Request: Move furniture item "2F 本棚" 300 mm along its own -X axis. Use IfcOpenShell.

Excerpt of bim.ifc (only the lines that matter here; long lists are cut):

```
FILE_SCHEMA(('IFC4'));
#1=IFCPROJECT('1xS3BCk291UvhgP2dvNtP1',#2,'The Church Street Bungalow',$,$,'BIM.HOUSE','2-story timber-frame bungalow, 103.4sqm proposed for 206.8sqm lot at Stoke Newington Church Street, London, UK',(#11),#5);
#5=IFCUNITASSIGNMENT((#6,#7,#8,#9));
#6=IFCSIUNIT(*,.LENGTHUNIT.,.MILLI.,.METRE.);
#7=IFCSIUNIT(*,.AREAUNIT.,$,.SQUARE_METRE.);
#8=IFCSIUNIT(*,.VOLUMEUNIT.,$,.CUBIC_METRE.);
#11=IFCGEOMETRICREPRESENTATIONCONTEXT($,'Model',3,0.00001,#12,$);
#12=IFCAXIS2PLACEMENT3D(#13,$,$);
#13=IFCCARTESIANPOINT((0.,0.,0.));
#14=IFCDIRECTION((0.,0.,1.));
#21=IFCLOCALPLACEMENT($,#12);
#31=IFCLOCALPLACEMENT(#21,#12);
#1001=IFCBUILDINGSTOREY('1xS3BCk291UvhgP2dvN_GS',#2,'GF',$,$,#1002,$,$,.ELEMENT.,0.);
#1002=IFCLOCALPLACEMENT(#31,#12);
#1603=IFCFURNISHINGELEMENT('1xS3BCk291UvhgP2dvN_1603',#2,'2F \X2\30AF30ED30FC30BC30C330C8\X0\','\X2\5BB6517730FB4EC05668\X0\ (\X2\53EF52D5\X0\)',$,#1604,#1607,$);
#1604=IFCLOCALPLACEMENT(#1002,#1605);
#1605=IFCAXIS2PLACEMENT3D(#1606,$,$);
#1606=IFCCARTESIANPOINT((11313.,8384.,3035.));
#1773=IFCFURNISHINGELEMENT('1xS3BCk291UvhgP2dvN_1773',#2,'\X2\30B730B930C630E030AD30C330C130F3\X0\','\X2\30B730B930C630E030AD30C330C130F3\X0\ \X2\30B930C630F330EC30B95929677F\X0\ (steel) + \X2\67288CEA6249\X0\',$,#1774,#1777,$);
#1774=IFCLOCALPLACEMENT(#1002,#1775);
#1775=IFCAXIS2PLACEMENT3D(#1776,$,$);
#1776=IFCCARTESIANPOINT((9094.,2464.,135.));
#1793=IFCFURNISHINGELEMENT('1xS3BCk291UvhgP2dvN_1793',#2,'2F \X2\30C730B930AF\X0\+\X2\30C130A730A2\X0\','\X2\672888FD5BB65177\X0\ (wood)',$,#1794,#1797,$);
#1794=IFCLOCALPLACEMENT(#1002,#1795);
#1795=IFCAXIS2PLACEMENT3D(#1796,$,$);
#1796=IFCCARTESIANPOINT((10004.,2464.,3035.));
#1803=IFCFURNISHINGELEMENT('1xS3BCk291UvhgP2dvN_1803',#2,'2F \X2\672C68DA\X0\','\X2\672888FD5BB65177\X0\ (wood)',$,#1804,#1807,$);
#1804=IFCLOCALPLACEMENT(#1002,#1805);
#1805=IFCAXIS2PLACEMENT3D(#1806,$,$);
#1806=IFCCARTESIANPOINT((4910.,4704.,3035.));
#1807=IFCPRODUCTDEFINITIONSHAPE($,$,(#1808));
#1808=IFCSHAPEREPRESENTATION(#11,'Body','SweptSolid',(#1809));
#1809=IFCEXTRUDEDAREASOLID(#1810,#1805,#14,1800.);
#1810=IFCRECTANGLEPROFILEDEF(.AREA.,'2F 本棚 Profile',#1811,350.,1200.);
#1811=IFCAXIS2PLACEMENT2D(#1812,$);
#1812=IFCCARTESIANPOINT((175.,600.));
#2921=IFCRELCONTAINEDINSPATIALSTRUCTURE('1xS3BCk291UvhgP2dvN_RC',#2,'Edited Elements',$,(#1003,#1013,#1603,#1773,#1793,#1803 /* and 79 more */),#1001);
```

```python
import ifcopenshell
import ifcopenshell.api.geometry
import ifcopenshell.util.placement
import ifcopenshell.util.unit

model = ifcopenshell.open("bim.ifc")
unit_scale = ifcopenshell.util.unit.calculate_unit_scale(model)

item = model.by_guid("1xS3BCk291UvhgP2dvN_1803")
matrix = ifcopenshell.util.placement.get_local_placement(item.ObjectPlacement)
matrix[:3, 3] -= matrix[:3, 0] * 0.3 / unit_scale
ifcopenshell.api.geometry.edit_object_placement(model, product=item, matrix=matrix, is_si=False)

print(ifcopenshell.util.placement.get_local_placement(item.ObjectPlacement).round(3) + 0.0)

model.write("bim-out.ifc")
```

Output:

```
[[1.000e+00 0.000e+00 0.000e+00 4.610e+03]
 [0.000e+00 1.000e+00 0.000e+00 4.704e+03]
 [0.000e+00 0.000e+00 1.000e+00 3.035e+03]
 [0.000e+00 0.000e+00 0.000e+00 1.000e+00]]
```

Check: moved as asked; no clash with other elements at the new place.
